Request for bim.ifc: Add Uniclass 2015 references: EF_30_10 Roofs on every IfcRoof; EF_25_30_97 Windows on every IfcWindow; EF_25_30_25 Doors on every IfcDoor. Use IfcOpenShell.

First a look at what the model holds.

```python
import ifcopenshell

model = ifcopenshell.open("bim.ifc")
print(model.schema)
print("classifications:", [c.Name for c in model.by_type("IfcClassification")])
for ifc_class in ("IfcDoor", "IfcRoof", "IfcStair", "IfcWall", "IfcWindow"):
    print(ifc_class, len(model.by_type(ifc_class)))
```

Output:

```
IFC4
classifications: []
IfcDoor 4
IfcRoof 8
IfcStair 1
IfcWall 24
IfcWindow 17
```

```python
import ifcopenshell
import ifcopenshell.api.classification

model = ifcopenshell.open("bim.ifc")

system = ifcopenshell.api.classification.add_classification(model, classification="Uniclass 2015")

codes = {
    "IfcRoof": ("EF_30_10", "Roofs"),
    "IfcWindow": ("EF_25_30_97", "Windows"),
    "IfcDoor": ("EF_25_30_25", "Doors"),
}
for ifc_class, (code, name) in codes.items():
    products = model.by_type(ifc_class)
    ifcopenshell.api.classification.add_reference(
        model, products=products, classification=system, identification=code, name=name
    )
    print(code, len(products))

model.write("bim_updated.ifc")
```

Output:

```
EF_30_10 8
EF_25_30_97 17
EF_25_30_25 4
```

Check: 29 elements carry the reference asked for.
